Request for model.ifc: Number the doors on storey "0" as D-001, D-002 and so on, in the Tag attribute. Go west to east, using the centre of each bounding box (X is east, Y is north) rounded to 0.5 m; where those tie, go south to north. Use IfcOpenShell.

First a look at what the model holds.

```python
import ifcopenshell
import ifcopenshell.util.element
import ifcopenshell.util.placement

model = ifcopenshell.open("model.ifc")
print(model.schema)
storey = next(s for s in model.by_type("IfcBuildingStorey") if s.Name == "0")
doors = [e for e in ifcopenshell.util.element.get_decomposition(storey) if e.is_a("IfcDoor")]
for e in sorted(doors, key=lambda e: e.id()):
    origin = ifcopenshell.util.placement.get_local_placement(e.ObjectPlacement)[:3, 3]
    print(e.id(), e.Tag, e.Name, origin.round(2) + 0.0, sep=" | ")
```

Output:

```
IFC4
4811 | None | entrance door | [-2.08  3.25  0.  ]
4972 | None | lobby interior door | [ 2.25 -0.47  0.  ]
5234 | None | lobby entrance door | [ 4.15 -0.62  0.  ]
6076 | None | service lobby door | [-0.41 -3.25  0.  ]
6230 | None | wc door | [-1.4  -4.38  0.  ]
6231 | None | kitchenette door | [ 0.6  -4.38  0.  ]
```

```python
import ifcopenshell
import ifcopenshell.geom
import ifcopenshell.util.element
import ifcopenshell.util.shape

model = ifcopenshell.open("model.ifc")
settings = ifcopenshell.geom.settings()
settings.set("use-world-coords", True)


def centre(element):
    shape = ifcopenshell.geom.create_shape(settings, element)
    return ifcopenshell.util.shape.get_bbox_centroid(shape.geometry)


storey = next(s for s in model.by_type("IfcBuildingStorey") if s.Name == "0")
doors = [e for e in ifcopenshell.util.element.get_decomposition(storey) if e.is_a("IfcDoor")]

# Insertion points can sit at a corner or the storey origin, so sort by the geometry (in metres).
centres = {e: centre(e) for e in doors}
doors.sort(key=lambda e: (round(centres[e][0] / 0.5), centres[e][1]))

for i, e in enumerate(doors, start=1):
    number = f"D-0{i:02d}"
    e.Tag = number
    print(e.id(), number)

model.write("model-out.ifc")
```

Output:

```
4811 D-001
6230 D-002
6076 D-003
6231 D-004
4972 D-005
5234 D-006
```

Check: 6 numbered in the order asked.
